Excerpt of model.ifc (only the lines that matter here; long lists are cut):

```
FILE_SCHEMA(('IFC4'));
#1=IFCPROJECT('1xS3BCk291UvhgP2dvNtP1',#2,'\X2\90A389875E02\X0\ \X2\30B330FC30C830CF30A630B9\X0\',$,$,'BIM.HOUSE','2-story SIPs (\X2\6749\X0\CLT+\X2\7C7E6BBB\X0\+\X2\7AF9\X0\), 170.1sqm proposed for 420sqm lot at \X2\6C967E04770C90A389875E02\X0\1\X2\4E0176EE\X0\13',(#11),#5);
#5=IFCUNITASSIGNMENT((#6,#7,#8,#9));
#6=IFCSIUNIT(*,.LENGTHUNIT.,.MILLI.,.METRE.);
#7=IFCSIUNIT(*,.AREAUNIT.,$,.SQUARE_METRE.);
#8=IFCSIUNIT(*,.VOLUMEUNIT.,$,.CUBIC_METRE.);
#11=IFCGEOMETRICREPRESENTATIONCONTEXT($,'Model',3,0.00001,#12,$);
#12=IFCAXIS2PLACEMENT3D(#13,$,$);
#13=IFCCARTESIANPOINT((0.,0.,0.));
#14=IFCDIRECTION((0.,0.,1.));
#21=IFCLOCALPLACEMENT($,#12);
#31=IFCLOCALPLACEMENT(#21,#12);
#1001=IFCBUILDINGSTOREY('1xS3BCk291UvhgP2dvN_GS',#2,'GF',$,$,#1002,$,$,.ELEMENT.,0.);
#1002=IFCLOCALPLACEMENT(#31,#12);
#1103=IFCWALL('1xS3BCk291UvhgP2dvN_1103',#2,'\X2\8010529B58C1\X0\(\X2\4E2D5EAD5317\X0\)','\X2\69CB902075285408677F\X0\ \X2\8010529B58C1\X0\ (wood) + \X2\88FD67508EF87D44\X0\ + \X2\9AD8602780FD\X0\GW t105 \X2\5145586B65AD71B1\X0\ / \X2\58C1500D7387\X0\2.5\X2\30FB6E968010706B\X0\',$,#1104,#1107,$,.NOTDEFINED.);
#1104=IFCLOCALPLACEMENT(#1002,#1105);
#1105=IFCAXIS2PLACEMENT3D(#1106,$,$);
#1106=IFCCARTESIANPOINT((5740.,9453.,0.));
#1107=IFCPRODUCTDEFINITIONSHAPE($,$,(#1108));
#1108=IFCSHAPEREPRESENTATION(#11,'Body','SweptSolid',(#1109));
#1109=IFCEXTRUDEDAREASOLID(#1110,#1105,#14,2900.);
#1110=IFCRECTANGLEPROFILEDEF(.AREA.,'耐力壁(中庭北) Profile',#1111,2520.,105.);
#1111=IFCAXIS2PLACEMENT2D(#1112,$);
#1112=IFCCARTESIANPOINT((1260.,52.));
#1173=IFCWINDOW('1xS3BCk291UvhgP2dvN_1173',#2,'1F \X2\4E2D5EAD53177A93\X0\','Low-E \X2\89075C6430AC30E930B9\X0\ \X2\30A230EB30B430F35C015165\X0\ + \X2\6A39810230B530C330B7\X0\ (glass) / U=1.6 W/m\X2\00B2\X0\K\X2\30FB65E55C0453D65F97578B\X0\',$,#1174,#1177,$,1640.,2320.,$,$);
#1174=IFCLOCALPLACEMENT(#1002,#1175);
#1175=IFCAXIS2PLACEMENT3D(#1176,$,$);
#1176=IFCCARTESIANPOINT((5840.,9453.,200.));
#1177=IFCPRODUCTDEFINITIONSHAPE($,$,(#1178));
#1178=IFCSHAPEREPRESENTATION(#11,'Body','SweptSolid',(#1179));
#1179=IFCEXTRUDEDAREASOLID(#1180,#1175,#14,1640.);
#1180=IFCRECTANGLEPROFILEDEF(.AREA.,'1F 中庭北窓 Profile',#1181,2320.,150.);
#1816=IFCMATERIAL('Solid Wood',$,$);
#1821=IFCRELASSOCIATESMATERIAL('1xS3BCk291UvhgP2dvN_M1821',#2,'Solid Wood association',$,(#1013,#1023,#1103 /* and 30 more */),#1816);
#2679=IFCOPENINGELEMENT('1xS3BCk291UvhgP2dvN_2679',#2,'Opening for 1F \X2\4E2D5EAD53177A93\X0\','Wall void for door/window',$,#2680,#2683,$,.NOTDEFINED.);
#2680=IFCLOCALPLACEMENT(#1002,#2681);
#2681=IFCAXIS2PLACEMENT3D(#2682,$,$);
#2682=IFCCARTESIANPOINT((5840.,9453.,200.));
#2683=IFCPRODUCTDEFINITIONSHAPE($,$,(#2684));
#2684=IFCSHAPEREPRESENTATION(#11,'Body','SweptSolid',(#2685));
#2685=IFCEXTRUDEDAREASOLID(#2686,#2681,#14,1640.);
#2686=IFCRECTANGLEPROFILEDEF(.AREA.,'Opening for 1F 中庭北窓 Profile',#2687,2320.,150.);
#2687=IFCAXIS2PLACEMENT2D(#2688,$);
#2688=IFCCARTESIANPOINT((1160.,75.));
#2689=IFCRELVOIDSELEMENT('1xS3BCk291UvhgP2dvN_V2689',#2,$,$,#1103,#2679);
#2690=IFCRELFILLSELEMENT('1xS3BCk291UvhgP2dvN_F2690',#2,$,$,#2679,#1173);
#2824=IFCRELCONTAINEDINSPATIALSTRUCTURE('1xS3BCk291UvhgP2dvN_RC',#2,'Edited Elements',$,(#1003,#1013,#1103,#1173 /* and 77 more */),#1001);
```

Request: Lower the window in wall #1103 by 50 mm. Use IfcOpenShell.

```python
import numpy as np
import ifcopenshell
import ifcopenshell.api.geometry
import ifcopenshell.util.placement
import ifcopenshell.util.unit

model = ifcopenshell.open("model.ifc")
unit_scale = ifcopenshell.util.unit.calculate_unit_scale(model)

window = model.by_guid("1xS3BCk291UvhgP2dvN_1173")
opening = window.FillsVoids[0].RelatingOpeningElement
dz = -50.0

shift = np.array([0.0, 0.0, dz])
# The window is not placed relative to its opening, so move both.
for product in (opening, window):
    matrix = ifcopenshell.util.placement.get_local_placement(product.ObjectPlacement)
    matrix[:3, 3] += shift
    ifcopenshell.api.geometry.edit_object_placement(model, product=product, matrix=matrix, is_si=False)

print(f"moved by {dz * unit_scale:+.3f} m")

model.write("model_rev.ifc")
```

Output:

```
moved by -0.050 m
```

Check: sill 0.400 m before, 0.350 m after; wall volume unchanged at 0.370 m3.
